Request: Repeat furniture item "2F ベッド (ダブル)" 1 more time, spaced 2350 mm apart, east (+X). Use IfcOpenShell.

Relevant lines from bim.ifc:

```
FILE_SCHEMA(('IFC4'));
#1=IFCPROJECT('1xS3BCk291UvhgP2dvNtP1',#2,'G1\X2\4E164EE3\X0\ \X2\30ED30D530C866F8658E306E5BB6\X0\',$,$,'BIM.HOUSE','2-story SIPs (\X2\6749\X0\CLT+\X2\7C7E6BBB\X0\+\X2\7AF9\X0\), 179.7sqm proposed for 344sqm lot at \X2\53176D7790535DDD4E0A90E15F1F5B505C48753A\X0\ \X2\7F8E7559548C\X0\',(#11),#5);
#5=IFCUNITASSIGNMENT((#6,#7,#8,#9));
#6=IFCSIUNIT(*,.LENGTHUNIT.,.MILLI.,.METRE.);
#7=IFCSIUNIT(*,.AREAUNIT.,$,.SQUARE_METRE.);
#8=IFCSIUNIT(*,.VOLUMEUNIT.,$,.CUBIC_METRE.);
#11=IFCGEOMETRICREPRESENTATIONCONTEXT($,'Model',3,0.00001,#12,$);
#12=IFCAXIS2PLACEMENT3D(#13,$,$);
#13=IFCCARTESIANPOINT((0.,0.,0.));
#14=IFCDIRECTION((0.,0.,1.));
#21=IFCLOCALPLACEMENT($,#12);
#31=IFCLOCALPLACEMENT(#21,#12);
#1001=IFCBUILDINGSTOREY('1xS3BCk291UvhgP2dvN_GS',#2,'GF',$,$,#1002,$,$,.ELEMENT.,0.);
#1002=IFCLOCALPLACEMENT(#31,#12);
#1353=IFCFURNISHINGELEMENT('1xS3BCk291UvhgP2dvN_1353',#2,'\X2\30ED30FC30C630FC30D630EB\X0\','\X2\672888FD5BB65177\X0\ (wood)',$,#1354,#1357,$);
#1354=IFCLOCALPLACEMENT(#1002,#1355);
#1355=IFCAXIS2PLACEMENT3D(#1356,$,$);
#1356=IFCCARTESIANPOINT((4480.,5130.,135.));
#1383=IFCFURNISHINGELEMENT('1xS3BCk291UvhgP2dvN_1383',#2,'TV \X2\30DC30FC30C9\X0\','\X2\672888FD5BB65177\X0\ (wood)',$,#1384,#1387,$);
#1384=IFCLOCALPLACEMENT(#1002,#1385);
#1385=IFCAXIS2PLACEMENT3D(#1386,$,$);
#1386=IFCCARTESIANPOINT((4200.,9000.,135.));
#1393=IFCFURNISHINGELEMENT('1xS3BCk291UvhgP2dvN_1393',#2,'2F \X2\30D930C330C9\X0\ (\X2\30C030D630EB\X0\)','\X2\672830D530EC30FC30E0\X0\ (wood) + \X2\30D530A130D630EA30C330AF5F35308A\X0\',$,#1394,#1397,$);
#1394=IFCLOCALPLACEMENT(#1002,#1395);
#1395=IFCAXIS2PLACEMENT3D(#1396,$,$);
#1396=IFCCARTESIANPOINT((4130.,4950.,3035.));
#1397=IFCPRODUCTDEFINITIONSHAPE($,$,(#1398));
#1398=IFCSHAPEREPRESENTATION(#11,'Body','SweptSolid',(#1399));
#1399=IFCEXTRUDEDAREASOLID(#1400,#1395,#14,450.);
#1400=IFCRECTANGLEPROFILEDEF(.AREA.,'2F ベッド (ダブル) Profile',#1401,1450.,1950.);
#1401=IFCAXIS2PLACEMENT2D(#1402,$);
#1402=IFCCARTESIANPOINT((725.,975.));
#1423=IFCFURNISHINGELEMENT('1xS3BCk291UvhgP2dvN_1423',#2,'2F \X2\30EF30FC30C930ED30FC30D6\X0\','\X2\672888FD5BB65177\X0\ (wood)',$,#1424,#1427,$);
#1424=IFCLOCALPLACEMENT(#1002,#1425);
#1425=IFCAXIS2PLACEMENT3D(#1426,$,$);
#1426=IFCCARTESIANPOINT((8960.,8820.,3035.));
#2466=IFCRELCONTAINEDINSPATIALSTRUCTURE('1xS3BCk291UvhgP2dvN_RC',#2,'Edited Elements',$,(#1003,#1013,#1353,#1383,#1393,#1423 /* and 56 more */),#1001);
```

```python
import numpy as np
import ifcopenshell
import ifcopenshell.api.geometry
import ifcopenshell.api.root
import ifcopenshell.util.element
import ifcopenshell.util.placement

model = ifcopenshell.open("bim.ifc")


def reuse_history(source, copy):
    """copy_class also copies each property set's owner history, people and application; keep the originals."""
    for rel in copy.IsDefinedBy:
        if rel.is_a("IfcRelDefinesByProperties") and (history := rel.RelatingPropertyDefinition.OwnerHistory):
            rel.RelatingPropertyDefinition.OwnerHistory = source.OwnerHistory
            ifcopenshell.util.element.remove_deep2(model, history)


source = model.by_id(1393)
base = ifcopenshell.util.placement.get_local_placement(source.ObjectPlacement)
step = np.array([1.0, 0.0, 0.0]) * 2350.0

for i in range(1, 2):
    copy = ifcopenshell.api.root.copy_class(model, product=source)
    copy.Representation = ifcopenshell.util.element.copy_deep(
        model, source.Representation, exclude=["IfcGeometricRepresentationContext", "IfcRepresentationMap"]
    )
    reuse_history(source, copy)
    matrix = base.copy()
    matrix[:3, 3] += i * step
    print("added at", matrix[:3, 3].round(3) + 0.0)
    ifcopenshell.api.geometry.edit_object_placement(model, product=copy, matrix=matrix, is_si=False)

model.write("bim_v2.ifc")
```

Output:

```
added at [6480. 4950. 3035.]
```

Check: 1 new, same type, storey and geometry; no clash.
